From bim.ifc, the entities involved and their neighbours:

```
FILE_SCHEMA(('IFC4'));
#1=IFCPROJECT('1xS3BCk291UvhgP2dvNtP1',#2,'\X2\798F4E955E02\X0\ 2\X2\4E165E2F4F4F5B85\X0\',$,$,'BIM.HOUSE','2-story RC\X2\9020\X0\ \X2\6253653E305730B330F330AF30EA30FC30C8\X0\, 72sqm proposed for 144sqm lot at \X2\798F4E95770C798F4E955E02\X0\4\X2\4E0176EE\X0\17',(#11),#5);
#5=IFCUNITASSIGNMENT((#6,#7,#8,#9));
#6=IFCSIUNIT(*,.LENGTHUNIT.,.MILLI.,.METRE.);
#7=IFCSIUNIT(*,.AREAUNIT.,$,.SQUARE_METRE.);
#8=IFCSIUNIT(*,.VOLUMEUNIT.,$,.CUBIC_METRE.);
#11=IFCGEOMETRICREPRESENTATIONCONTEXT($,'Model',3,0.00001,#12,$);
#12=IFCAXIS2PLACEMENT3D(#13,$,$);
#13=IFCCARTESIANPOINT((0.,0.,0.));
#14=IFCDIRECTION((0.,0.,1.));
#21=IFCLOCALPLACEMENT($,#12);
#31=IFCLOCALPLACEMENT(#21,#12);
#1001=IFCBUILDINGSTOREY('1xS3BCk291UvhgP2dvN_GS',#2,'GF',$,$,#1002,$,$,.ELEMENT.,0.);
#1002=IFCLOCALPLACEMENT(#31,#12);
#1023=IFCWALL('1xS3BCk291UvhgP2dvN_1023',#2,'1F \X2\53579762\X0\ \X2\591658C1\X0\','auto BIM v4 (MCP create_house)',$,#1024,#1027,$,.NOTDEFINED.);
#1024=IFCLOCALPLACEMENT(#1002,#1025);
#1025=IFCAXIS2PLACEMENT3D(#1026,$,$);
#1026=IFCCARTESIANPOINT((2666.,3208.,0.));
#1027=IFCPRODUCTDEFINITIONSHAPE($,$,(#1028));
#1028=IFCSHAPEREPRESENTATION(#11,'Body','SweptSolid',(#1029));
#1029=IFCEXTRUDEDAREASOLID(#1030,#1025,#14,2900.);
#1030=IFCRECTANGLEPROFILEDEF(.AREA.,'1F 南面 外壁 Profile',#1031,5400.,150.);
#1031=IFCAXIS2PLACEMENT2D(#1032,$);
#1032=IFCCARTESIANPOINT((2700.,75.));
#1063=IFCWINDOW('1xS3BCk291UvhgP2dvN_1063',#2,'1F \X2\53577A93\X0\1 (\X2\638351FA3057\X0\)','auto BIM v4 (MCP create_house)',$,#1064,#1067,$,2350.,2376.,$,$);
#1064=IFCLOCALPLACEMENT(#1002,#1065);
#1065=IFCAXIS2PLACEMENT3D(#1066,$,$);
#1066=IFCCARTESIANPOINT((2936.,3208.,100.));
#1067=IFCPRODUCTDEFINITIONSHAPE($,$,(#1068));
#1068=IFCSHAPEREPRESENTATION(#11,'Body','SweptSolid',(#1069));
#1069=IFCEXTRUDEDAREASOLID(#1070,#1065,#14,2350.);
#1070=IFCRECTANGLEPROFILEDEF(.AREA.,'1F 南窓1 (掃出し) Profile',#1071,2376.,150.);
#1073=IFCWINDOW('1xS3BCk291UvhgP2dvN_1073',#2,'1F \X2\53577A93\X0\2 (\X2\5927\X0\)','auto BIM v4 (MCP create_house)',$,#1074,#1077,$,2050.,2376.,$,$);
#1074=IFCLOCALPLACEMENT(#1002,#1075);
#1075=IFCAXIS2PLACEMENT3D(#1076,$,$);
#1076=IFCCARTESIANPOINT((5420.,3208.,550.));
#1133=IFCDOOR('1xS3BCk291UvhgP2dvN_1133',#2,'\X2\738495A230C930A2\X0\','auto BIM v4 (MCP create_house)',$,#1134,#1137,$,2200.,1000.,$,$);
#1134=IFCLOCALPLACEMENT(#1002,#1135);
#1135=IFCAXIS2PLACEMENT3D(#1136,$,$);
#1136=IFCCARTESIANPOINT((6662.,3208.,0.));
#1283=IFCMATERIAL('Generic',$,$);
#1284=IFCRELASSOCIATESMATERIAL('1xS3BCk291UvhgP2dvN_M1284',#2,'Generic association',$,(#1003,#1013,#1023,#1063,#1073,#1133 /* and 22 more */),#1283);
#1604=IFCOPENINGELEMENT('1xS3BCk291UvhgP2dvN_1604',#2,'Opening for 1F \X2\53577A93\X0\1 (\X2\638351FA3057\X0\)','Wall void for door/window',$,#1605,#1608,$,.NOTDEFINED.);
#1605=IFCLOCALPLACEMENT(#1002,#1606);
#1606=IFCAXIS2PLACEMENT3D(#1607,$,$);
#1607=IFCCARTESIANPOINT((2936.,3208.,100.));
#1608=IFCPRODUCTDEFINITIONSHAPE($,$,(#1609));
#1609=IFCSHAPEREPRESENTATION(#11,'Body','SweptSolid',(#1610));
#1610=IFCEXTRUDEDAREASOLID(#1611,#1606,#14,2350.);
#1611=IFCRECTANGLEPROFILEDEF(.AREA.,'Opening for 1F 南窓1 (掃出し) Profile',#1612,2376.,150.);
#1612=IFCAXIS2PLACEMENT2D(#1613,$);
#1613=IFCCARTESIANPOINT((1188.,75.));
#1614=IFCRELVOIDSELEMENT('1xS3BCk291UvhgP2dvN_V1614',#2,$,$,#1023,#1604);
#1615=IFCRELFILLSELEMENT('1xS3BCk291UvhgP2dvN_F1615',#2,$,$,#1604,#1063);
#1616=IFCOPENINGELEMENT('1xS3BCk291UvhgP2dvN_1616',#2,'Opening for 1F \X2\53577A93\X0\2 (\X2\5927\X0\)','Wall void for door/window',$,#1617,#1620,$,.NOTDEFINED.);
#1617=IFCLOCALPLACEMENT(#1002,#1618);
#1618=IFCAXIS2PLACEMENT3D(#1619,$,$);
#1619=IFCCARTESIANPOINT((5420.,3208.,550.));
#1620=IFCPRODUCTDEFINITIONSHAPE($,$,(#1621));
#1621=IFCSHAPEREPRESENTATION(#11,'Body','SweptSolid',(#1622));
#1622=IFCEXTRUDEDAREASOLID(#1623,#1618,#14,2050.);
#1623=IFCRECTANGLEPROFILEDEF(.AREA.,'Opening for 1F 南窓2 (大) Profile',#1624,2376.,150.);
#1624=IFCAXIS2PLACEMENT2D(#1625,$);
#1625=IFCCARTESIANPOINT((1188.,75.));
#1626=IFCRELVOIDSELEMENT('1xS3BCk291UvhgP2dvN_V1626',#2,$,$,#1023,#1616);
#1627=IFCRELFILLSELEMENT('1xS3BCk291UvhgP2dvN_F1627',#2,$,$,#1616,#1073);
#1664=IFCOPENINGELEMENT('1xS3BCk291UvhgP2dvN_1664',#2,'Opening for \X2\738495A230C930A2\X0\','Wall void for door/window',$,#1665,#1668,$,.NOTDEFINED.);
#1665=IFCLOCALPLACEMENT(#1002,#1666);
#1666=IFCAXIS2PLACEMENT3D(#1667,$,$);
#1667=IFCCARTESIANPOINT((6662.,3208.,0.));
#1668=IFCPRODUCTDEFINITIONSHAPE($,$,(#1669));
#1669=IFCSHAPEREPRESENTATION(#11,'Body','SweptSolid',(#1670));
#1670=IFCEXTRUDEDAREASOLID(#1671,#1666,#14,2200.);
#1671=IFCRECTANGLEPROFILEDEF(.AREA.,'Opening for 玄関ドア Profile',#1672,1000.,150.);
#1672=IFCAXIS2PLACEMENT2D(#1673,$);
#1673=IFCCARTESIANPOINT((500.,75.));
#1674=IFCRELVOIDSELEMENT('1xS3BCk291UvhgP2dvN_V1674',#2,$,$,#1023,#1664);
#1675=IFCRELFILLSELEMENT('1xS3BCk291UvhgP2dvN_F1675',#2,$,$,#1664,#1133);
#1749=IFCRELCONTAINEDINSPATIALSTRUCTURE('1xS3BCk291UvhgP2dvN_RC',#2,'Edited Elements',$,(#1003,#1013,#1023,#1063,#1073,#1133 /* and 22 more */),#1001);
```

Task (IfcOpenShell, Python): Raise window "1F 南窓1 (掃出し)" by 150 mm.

```python
import numpy as np
import ifcopenshell
import ifcopenshell.api.geometry
import ifcopenshell.util.placement
import ifcopenshell.util.unit

model = ifcopenshell.open("bim.ifc")
unit_scale = ifcopenshell.util.unit.calculate_unit_scale(model)

window = model.by_guid("1xS3BCk291UvhgP2dvN_1063")
opening = window.FillsVoids[0].RelatingOpeningElement
dz = 150.0

shift = np.array([0.0, 0.0, dz])
# The window is not placed relative to its opening, so move both.
for product in (opening, window):
    matrix = ifcopenshell.util.placement.get_local_placement(product.ObjectPlacement)
    matrix[:3, 3] += shift
    ifcopenshell.api.geometry.edit_object_placement(model, product=product, matrix=matrix, is_si=False)

print(f"moved by {dz * unit_scale:+.3f} m")

model.write("bim-out.ifc")
```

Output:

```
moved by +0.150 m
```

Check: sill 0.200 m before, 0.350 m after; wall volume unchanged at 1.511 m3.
